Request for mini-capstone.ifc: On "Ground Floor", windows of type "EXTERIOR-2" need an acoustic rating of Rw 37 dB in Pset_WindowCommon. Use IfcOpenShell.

First a look at what the model holds.

```python
import ifcopenshell
import ifcopenshell.util.element

model = ifcopenshell.open("mini-capstone.ifc")
print(model.schema)
storey = next(s for s in model.by_type("IfcBuildingStorey") if s.Name == "Ground Floor")
windows = [e for e in ifcopenshell.util.element.get_decomposition(storey) if e.is_a("IfcWindow")]
seen = {}
for e in windows:
    element_type = ifcopenshell.util.element.get_type(e)
    key = (element_type.Name if element_type != e and element_type else None, ifcopenshell.util.element.get_pset(e, "Pset_WindowCommon", "AcousticRating"))
    seen[key] = seen.get(key, 0) + 1
for (name, value), count in sorted(seen.items(), key=str):
    print(count, "x", name, "|", value)
```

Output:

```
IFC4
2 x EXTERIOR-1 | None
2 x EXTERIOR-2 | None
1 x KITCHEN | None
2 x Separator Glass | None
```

```python
import ifcopenshell
import ifcopenshell.api.pset
import ifcopenshell.util.element

model = ifcopenshell.open("mini-capstone.ifc")

storey = next(s for s in model.by_type("IfcBuildingStorey") if s.Name == "Ground Floor")
windows = [e for e in ifcopenshell.util.element.get_decomposition(storey) if e.is_a("IfcWindow")]

count = 0
for e in windows:
    element_type = ifcopenshell.util.element.get_type(e)
    if element_type in (None, e) or element_type.Name != "EXTERIOR-2":
        continue
    # add_pset returns the element's existing set when there is one.
    pset = ifcopenshell.api.pset.add_pset(model, product=e, name="Pset_WindowCommon")
    ifcopenshell.api.pset.edit_pset(model, pset=pset, properties={"AcousticRating": "Rw 37 dB"})
    count += 1

print(count, "windows updated")

model.write("mini-capstone_rev.ifc")
```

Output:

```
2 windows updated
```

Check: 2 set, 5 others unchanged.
